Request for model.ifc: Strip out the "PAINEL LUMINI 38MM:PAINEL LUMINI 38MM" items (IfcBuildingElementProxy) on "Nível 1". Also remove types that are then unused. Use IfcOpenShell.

First a look at what the model holds.

```python
import ifcopenshell
import ifcopenshell.util.element

model = ifcopenshell.open("model.ifc")
print(model.schema)
storey = next(s for s in model.by_type("IfcBuildingStorey") if s.Name == "Nível 1")
proxies = [e for e in ifcopenshell.util.element.get_decomposition(storey) if e.is_a("IfcBuildingElementProxy")]
seen = {}
for e in proxies:
    element_type = ifcopenshell.util.element.get_type(e)
    name = element_type.Name if element_type not in (None, e) else None
    seen[name] = seen.get(name, 0) + 1
for name, count in sorted(seen.items(), key=str):
    print(count, "x", name)
```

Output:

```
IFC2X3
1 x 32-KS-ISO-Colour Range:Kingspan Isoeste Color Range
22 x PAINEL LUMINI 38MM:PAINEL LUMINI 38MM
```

```python
import ifcopenshell
import ifcopenshell.api.root
import ifcopenshell.util.element

model = ifcopenshell.open("model.ifc")

storey = next(s for s in model.by_type("IfcBuildingStorey") if s.Name == "Nível 1")
proxies = [e for e in ifcopenshell.util.element.get_decomposition(storey) if e.is_a("IfcBuildingElementProxy")]
targets = [e for e in proxies if (t := ifcopenshell.util.element.get_type(e)) not in (None, e) and t.Name == "PAINEL LUMINI 38MM:PAINEL LUMINI 38MM"]
types = {ifcopenshell.util.element.get_type(e) for e in targets} - {None, *targets}

for e in targets:
    ifcopenshell.api.root.remove_product(model, product=e)
print(len(targets), "removed")

unused = [t for t in types if not ifcopenshell.util.element.get_types(t)]
for t in unused:
    ifcopenshell.api.root.remove_product(model, product=t)
print(len(unused), "unused types removed")

model.write("model_rev.ifc")
```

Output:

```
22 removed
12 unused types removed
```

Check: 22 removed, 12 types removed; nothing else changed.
